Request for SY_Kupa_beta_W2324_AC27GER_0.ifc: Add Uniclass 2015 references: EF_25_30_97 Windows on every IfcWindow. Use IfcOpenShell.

First a look at what the model holds.

```python
import ifcopenshell

model = ifcopenshell.open("SY_Kupa_beta_W2324_AC27GER_0.ifc")
print(model.schema)
print("classifications:", [c.Name for c in model.by_type("IfcClassification")])
for ifc_class in ("IfcDoor", "IfcRoof", "IfcStair", "IfcWall", "IfcWindow"):
    print(ifc_class, len(model.by_type(ifc_class)))
```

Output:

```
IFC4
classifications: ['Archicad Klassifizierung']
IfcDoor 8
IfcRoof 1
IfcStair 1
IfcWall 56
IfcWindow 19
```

```python
import ifcopenshell
import ifcopenshell.api.classification

model = ifcopenshell.open("SY_Kupa_beta_W2324_AC27GER_0.ifc")

system = ifcopenshell.api.classification.add_classification(model, classification="Uniclass 2015")

codes = {
    "IfcWindow": ("EF_25_30_97", "Windows"),
}
for ifc_class, (code, name) in codes.items():
    products = model.by_type(ifc_class)
    ifcopenshell.api.classification.add_reference(
        model, products=products, classification=system, identification=code, name=name
    )
    print(code, len(products))

model.write("SY_Kupa_beta_W2324_AC27GER_0-out.ifc")
```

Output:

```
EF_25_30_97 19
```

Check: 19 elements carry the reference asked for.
